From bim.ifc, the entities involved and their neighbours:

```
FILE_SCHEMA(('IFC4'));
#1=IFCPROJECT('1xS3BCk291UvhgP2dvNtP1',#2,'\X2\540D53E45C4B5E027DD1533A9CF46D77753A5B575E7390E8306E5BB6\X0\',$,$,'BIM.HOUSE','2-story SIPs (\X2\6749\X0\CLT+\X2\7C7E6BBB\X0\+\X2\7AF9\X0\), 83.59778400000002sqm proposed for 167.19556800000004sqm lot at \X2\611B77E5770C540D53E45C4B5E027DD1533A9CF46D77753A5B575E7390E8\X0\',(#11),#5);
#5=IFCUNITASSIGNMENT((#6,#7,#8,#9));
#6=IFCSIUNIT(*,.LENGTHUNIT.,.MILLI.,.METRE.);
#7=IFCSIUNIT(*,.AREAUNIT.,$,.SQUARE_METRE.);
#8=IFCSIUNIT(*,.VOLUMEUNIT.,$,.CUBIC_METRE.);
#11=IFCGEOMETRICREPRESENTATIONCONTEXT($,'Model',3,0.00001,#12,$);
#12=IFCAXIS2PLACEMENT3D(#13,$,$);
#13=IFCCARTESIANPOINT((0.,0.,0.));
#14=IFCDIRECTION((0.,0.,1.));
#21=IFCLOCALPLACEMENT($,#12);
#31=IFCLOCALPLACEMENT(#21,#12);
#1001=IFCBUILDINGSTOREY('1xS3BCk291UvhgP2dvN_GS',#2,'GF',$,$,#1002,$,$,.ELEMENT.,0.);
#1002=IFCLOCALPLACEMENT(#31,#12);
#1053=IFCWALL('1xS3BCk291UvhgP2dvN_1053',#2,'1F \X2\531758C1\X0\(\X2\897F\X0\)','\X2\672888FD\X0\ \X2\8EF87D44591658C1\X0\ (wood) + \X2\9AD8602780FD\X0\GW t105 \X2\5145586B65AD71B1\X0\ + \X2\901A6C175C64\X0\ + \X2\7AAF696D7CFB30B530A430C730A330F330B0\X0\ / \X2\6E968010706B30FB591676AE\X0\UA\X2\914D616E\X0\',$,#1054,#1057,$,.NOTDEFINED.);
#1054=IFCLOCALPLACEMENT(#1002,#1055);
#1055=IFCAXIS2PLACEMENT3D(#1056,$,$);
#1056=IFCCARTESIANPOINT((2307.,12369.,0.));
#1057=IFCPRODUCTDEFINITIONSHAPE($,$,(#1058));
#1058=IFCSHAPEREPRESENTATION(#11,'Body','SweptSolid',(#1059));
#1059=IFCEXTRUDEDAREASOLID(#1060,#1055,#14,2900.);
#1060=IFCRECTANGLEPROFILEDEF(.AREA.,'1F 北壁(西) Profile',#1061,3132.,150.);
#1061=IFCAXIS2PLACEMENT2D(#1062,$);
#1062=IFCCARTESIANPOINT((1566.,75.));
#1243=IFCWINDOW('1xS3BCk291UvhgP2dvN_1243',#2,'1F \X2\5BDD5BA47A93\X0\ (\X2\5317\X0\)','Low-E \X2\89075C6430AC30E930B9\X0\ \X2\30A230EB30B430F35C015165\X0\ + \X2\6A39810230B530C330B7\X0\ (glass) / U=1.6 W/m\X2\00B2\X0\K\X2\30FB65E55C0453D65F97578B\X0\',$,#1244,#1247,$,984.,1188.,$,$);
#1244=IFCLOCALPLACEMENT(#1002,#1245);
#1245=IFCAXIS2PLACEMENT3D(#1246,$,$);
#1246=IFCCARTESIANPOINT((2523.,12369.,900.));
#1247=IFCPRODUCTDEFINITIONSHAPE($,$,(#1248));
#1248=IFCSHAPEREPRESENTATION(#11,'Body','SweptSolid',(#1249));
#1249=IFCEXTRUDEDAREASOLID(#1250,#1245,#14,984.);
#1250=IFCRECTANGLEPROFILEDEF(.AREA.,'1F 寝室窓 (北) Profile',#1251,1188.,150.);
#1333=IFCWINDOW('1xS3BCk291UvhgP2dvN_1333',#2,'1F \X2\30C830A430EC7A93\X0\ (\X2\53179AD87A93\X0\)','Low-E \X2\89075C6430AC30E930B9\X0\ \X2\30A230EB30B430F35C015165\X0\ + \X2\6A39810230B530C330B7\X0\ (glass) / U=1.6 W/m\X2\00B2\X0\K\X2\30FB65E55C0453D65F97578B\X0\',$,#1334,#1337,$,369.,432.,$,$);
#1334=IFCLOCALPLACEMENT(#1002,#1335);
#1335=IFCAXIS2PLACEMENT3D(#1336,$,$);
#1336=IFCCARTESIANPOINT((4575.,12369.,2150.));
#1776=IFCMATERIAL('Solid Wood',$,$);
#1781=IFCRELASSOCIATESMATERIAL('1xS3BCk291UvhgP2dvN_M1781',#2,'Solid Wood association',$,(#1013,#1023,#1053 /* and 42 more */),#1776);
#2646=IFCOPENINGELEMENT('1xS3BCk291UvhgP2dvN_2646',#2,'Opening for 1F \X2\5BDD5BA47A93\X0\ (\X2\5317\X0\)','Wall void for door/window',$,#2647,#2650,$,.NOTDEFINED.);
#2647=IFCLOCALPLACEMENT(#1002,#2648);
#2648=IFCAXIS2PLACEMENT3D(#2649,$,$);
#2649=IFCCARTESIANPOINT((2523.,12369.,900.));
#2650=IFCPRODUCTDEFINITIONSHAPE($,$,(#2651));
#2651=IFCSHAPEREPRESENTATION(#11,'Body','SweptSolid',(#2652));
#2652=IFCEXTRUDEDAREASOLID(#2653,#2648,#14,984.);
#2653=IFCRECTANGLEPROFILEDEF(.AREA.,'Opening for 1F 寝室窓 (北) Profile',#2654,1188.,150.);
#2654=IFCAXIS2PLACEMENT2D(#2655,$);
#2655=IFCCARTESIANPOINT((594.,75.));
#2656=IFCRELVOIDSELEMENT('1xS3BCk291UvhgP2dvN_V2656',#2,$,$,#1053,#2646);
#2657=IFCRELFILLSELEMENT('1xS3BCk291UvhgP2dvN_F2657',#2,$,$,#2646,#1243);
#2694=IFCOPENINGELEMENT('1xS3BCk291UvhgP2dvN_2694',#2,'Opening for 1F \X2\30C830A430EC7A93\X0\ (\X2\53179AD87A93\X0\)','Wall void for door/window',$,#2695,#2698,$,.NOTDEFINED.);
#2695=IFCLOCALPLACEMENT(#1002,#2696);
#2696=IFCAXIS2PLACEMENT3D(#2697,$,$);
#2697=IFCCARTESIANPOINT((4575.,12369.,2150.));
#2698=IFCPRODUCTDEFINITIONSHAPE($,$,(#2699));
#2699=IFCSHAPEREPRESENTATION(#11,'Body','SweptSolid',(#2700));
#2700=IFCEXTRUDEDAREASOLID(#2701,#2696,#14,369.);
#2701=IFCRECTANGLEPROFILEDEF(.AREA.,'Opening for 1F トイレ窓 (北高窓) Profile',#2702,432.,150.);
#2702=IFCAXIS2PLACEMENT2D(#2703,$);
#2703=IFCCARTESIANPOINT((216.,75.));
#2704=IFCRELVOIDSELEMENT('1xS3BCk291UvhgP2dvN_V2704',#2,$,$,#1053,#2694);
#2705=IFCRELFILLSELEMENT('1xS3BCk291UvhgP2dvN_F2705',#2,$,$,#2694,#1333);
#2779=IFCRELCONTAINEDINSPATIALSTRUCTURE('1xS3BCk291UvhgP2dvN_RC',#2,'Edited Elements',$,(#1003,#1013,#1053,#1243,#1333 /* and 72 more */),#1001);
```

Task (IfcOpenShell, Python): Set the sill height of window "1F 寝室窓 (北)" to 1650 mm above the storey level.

```python
import numpy as np
import ifcopenshell
import ifcopenshell.api.geometry
import ifcopenshell.geom
import ifcopenshell.util.element
import ifcopenshell.util.placement
import ifcopenshell.util.shape
import ifcopenshell.util.unit

model = ifcopenshell.open("bim.ifc")
unit_scale = ifcopenshell.util.unit.calculate_unit_scale(model)

window = model.by_guid("1xS3BCk291UvhgP2dvN_1243")
opening = window.FillsVoids[0].RelatingOpeningElement
storey = ifcopenshell.util.element.get_container(window, ifc_class="IfcBuildingStorey")
level = ifcopenshell.util.placement.get_local_placement(storey.ObjectPlacement)[2, 3]

# The opening's origin need not be at the sill, so measure its lowest point.
shape = ifcopenshell.geom.create_shape(ifcopenshell.geom.settings(), opening)
bottom = ifcopenshell.util.shape.get_shape_bottom_elevation(shape, shape.geometry) / unit_scale
dz = level + 1650.0 - bottom

shift = np.array([0.0, 0.0, dz])
# The window is not placed relative to its opening, so move both.
for product in (opening, window):
    matrix = ifcopenshell.util.placement.get_local_placement(product.ObjectPlacement)
    matrix[:3, 3] += shift
    ifcopenshell.api.geometry.edit_object_placement(model, product=product, matrix=matrix, is_si=False)

print(f"moved by {dz * unit_scale:+.3f} m")

model.write("bim_rev.ifc")
```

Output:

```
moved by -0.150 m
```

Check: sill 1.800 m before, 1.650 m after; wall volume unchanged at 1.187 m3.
